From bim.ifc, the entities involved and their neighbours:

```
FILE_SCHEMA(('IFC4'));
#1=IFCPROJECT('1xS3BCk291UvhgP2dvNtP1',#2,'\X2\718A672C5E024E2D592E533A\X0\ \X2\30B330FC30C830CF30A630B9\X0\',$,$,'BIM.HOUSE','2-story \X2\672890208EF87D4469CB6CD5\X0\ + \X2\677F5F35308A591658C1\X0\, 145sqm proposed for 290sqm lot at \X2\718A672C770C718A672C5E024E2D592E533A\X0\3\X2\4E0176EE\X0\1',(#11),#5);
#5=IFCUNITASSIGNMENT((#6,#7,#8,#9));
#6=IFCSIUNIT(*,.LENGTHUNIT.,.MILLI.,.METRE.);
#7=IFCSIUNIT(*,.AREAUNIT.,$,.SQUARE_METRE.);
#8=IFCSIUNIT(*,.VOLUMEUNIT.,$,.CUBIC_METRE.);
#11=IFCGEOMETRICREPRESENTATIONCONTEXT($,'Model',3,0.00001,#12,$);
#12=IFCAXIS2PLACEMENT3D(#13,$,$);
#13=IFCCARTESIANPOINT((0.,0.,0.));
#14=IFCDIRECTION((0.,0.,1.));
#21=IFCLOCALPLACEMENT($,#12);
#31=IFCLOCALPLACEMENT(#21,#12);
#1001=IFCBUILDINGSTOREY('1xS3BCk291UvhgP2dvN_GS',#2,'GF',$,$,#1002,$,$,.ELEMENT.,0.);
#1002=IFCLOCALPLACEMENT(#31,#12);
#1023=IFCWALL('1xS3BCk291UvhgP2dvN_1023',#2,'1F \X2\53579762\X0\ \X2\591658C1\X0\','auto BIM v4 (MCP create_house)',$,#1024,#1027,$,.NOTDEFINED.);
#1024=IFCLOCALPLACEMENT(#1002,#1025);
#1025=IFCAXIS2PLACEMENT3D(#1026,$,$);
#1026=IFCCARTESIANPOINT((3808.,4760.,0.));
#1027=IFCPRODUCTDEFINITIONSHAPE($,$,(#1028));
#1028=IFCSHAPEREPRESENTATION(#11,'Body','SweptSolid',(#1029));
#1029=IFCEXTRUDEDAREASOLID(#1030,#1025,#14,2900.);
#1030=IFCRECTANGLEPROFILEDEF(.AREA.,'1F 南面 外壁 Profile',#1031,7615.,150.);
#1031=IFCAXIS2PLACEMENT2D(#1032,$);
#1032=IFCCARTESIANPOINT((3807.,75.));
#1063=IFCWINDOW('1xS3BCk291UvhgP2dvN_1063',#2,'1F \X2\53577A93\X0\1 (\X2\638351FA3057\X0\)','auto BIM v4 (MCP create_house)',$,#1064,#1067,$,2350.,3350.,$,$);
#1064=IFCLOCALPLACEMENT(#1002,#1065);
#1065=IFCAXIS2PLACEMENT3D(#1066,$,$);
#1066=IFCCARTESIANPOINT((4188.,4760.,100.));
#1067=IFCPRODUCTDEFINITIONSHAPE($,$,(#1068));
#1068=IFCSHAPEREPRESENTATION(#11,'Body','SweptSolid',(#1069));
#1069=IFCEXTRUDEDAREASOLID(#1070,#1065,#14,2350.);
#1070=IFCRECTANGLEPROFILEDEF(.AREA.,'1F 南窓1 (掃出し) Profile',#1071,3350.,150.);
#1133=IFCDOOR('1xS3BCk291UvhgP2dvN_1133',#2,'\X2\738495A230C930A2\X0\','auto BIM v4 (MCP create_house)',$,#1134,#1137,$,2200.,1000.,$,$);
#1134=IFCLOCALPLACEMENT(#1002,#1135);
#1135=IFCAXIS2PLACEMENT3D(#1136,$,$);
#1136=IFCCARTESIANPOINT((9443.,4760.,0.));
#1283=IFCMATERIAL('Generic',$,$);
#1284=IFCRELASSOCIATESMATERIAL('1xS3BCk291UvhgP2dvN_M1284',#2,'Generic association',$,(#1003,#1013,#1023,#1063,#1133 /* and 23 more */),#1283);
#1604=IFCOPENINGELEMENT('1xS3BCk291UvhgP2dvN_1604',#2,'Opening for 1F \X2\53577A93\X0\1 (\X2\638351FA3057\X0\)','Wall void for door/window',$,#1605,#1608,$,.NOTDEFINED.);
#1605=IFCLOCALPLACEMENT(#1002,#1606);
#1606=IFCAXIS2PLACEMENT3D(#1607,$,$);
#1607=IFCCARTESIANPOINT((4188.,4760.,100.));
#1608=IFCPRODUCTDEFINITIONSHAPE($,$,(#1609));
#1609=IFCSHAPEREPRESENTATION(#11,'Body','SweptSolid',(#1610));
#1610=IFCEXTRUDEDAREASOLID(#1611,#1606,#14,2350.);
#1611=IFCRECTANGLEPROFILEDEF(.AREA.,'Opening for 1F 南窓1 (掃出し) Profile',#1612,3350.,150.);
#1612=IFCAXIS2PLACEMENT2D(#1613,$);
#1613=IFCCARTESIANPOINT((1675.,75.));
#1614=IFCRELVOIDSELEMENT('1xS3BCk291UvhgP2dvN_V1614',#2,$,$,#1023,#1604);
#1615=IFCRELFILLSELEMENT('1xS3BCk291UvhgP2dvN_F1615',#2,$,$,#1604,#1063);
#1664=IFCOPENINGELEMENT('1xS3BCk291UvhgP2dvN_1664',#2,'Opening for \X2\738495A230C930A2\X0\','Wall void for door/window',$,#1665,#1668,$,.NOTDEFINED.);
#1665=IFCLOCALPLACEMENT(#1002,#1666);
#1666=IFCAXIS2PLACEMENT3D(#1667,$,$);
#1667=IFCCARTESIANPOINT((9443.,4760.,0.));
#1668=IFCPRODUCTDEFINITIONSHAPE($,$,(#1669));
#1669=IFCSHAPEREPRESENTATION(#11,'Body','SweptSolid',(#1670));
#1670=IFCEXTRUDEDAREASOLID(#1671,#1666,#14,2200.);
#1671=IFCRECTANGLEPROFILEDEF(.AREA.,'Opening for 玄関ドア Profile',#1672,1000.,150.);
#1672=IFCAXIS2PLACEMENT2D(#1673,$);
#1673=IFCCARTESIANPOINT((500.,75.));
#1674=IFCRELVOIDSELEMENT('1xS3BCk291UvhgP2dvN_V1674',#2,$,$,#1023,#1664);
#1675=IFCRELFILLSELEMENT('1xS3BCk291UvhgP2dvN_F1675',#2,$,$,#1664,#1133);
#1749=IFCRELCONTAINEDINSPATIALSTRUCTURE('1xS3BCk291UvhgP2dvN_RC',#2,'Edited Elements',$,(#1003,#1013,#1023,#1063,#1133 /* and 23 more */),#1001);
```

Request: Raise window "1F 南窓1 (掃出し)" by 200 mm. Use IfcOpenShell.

```python
import numpy as np
import ifcopenshell
import ifcopenshell.api.geometry
import ifcopenshell.util.placement
import ifcopenshell.util.unit

model = ifcopenshell.open("bim.ifc")
unit_scale = ifcopenshell.util.unit.calculate_unit_scale(model)

window = model.by_guid("1xS3BCk291UvhgP2dvN_1063")
opening = window.FillsVoids[0].RelatingOpeningElement
dz = 200.0

shift = np.array([0.0, 0.0, dz])
# The window is not placed relative to its opening, so move both.
for product in (opening, window):
    matrix = ifcopenshell.util.placement.get_local_placement(product.ObjectPlacement)
    matrix[:3, 3] += shift
    ifcopenshell.api.geometry.edit_object_placement(model, product=product, matrix=matrix, is_si=False)

print(f"moved by {dz * unit_scale:+.3f} m")

model.write("bim_v2.ifc")
```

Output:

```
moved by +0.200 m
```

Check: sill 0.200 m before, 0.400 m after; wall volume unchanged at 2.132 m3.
